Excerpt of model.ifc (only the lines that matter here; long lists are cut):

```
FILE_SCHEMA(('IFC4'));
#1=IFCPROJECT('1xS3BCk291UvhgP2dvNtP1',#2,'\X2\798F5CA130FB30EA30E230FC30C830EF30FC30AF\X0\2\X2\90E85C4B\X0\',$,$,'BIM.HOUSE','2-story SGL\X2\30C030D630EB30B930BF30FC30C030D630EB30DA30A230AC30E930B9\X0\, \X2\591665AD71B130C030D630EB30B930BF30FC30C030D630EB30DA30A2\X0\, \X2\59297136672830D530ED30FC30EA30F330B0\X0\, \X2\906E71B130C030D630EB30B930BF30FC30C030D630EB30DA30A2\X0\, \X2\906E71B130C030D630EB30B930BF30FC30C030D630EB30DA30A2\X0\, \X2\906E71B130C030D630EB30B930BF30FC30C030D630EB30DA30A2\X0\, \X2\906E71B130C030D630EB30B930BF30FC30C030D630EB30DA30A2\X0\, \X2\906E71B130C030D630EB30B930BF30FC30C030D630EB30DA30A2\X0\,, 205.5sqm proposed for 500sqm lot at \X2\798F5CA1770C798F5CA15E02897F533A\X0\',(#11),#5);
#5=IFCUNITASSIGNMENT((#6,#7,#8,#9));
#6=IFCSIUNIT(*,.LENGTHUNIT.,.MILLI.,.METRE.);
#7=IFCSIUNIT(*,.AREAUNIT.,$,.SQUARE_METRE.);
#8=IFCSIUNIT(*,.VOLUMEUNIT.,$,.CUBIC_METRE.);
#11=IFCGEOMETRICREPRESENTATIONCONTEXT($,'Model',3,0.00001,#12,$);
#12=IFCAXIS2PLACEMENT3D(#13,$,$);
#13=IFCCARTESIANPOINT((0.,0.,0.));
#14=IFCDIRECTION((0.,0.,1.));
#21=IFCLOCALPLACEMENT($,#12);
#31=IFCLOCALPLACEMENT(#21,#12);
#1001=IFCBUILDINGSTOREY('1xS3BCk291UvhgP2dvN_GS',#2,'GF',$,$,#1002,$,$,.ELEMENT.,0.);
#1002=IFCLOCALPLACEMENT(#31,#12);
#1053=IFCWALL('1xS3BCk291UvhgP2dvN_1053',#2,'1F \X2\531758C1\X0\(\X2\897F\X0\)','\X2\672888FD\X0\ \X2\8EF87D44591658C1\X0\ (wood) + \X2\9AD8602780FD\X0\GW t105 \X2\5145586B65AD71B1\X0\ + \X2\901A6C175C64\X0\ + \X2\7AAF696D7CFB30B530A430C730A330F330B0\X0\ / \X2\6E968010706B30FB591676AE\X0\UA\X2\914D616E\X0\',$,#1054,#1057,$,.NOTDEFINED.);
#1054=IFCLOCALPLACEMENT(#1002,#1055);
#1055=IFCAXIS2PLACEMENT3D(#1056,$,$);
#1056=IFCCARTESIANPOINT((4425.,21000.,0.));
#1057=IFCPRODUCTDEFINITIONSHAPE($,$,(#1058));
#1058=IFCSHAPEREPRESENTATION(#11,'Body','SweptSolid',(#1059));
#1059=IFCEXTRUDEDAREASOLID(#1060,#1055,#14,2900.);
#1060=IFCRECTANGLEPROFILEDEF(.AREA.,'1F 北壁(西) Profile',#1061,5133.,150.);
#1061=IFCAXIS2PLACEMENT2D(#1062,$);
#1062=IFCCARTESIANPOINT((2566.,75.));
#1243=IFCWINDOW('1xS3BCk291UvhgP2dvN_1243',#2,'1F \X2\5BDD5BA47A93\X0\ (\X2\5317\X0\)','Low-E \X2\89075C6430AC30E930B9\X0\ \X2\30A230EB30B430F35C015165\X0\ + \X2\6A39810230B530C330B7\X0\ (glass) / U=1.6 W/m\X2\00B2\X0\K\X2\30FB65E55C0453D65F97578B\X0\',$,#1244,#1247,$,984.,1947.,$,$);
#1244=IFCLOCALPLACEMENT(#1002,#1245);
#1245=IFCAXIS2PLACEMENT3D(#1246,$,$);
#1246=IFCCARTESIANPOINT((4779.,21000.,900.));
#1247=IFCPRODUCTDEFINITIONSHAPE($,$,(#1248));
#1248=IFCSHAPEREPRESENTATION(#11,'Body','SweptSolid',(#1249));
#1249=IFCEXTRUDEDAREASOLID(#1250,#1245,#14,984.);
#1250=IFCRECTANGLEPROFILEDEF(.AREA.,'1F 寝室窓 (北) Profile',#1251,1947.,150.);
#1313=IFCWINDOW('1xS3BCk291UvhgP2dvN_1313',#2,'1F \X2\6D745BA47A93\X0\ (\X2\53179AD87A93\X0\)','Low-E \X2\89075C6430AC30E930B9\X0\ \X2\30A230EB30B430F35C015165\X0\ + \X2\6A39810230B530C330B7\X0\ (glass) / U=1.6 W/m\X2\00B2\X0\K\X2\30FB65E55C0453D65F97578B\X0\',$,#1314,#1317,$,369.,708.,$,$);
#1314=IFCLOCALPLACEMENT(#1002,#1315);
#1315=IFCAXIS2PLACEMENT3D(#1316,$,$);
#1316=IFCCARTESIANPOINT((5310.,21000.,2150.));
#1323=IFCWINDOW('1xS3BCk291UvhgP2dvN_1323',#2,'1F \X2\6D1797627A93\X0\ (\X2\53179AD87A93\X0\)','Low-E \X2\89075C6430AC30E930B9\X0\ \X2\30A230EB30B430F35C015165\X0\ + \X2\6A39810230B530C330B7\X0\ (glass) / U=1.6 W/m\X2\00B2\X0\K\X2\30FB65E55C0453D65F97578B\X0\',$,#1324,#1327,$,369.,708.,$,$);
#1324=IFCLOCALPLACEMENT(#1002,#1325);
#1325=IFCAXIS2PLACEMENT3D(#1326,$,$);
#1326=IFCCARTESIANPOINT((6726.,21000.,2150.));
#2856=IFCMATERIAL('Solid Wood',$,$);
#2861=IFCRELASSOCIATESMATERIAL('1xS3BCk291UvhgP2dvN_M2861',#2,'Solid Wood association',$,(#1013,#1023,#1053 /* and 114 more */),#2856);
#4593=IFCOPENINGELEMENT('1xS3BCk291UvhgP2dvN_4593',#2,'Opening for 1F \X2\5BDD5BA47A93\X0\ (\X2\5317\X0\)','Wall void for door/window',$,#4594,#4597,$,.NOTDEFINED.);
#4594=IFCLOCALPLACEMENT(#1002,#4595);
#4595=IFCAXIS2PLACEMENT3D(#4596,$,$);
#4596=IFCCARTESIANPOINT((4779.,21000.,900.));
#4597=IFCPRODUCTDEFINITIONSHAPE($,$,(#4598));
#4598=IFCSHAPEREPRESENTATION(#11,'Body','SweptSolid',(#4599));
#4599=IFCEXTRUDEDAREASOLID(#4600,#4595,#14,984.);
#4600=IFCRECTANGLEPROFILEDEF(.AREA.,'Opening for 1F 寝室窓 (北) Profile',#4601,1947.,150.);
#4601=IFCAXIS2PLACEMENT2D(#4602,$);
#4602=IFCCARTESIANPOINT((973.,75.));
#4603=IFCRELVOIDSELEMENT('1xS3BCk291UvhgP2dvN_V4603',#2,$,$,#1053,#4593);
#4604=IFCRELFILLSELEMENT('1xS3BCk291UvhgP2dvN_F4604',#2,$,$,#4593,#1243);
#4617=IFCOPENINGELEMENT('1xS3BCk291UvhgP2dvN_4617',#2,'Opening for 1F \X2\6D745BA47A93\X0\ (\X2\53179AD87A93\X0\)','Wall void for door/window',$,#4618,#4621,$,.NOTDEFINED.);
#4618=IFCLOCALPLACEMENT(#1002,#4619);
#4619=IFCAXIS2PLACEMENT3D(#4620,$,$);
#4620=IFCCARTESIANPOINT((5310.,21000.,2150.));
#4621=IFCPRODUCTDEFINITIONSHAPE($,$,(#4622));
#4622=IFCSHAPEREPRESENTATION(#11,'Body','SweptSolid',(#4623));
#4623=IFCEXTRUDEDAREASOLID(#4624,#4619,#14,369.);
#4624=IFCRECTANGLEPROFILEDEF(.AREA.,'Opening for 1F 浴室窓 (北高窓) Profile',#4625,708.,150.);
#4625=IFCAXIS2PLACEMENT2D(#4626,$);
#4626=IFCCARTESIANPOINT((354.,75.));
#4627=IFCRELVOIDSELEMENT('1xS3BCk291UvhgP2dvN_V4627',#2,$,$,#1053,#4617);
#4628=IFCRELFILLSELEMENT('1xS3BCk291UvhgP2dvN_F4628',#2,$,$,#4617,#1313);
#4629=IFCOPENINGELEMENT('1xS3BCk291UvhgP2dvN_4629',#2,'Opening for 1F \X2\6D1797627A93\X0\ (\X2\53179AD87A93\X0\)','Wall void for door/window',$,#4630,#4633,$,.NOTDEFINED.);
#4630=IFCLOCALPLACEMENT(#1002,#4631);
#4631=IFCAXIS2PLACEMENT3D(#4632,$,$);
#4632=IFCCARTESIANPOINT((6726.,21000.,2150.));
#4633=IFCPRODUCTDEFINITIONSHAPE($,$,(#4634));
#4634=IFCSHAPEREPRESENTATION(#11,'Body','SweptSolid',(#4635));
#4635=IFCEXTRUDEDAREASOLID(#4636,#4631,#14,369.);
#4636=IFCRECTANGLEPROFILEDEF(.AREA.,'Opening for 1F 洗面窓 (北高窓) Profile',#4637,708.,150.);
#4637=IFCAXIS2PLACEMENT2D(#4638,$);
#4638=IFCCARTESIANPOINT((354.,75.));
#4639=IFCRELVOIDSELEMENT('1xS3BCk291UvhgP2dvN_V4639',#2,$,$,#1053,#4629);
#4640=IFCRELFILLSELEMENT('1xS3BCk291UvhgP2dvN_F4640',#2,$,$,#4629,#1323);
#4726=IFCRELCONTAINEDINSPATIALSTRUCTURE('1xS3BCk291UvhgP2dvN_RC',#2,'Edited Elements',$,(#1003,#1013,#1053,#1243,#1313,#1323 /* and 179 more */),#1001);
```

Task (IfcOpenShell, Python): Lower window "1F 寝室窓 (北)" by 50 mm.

```python
import numpy as np
import ifcopenshell
import ifcopenshell.api.geometry
import ifcopenshell.util.placement
import ifcopenshell.util.unit

model = ifcopenshell.open("model.ifc")
unit_scale = ifcopenshell.util.unit.calculate_unit_scale(model)

window = model.by_guid("1xS3BCk291UvhgP2dvN_1243")
opening = window.FillsVoids[0].RelatingOpeningElement
dz = -0.05 / unit_scale

shift = np.array([0.0, 0.0, dz])
# The window is not placed relative to its opening, so move both.
for product in (opening, window):
    matrix = ifcopenshell.util.placement.get_local_placement(product.ObjectPlacement)
    matrix[:3, 3] += shift
    ifcopenshell.api.geometry.edit_object_placement(model, product=product, matrix=matrix, is_si=False)

print(f"moved by {dz * unit_scale:+.3f} m")

model.write("model_edited.ifc")
```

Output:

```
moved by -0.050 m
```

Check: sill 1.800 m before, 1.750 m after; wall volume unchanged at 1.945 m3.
